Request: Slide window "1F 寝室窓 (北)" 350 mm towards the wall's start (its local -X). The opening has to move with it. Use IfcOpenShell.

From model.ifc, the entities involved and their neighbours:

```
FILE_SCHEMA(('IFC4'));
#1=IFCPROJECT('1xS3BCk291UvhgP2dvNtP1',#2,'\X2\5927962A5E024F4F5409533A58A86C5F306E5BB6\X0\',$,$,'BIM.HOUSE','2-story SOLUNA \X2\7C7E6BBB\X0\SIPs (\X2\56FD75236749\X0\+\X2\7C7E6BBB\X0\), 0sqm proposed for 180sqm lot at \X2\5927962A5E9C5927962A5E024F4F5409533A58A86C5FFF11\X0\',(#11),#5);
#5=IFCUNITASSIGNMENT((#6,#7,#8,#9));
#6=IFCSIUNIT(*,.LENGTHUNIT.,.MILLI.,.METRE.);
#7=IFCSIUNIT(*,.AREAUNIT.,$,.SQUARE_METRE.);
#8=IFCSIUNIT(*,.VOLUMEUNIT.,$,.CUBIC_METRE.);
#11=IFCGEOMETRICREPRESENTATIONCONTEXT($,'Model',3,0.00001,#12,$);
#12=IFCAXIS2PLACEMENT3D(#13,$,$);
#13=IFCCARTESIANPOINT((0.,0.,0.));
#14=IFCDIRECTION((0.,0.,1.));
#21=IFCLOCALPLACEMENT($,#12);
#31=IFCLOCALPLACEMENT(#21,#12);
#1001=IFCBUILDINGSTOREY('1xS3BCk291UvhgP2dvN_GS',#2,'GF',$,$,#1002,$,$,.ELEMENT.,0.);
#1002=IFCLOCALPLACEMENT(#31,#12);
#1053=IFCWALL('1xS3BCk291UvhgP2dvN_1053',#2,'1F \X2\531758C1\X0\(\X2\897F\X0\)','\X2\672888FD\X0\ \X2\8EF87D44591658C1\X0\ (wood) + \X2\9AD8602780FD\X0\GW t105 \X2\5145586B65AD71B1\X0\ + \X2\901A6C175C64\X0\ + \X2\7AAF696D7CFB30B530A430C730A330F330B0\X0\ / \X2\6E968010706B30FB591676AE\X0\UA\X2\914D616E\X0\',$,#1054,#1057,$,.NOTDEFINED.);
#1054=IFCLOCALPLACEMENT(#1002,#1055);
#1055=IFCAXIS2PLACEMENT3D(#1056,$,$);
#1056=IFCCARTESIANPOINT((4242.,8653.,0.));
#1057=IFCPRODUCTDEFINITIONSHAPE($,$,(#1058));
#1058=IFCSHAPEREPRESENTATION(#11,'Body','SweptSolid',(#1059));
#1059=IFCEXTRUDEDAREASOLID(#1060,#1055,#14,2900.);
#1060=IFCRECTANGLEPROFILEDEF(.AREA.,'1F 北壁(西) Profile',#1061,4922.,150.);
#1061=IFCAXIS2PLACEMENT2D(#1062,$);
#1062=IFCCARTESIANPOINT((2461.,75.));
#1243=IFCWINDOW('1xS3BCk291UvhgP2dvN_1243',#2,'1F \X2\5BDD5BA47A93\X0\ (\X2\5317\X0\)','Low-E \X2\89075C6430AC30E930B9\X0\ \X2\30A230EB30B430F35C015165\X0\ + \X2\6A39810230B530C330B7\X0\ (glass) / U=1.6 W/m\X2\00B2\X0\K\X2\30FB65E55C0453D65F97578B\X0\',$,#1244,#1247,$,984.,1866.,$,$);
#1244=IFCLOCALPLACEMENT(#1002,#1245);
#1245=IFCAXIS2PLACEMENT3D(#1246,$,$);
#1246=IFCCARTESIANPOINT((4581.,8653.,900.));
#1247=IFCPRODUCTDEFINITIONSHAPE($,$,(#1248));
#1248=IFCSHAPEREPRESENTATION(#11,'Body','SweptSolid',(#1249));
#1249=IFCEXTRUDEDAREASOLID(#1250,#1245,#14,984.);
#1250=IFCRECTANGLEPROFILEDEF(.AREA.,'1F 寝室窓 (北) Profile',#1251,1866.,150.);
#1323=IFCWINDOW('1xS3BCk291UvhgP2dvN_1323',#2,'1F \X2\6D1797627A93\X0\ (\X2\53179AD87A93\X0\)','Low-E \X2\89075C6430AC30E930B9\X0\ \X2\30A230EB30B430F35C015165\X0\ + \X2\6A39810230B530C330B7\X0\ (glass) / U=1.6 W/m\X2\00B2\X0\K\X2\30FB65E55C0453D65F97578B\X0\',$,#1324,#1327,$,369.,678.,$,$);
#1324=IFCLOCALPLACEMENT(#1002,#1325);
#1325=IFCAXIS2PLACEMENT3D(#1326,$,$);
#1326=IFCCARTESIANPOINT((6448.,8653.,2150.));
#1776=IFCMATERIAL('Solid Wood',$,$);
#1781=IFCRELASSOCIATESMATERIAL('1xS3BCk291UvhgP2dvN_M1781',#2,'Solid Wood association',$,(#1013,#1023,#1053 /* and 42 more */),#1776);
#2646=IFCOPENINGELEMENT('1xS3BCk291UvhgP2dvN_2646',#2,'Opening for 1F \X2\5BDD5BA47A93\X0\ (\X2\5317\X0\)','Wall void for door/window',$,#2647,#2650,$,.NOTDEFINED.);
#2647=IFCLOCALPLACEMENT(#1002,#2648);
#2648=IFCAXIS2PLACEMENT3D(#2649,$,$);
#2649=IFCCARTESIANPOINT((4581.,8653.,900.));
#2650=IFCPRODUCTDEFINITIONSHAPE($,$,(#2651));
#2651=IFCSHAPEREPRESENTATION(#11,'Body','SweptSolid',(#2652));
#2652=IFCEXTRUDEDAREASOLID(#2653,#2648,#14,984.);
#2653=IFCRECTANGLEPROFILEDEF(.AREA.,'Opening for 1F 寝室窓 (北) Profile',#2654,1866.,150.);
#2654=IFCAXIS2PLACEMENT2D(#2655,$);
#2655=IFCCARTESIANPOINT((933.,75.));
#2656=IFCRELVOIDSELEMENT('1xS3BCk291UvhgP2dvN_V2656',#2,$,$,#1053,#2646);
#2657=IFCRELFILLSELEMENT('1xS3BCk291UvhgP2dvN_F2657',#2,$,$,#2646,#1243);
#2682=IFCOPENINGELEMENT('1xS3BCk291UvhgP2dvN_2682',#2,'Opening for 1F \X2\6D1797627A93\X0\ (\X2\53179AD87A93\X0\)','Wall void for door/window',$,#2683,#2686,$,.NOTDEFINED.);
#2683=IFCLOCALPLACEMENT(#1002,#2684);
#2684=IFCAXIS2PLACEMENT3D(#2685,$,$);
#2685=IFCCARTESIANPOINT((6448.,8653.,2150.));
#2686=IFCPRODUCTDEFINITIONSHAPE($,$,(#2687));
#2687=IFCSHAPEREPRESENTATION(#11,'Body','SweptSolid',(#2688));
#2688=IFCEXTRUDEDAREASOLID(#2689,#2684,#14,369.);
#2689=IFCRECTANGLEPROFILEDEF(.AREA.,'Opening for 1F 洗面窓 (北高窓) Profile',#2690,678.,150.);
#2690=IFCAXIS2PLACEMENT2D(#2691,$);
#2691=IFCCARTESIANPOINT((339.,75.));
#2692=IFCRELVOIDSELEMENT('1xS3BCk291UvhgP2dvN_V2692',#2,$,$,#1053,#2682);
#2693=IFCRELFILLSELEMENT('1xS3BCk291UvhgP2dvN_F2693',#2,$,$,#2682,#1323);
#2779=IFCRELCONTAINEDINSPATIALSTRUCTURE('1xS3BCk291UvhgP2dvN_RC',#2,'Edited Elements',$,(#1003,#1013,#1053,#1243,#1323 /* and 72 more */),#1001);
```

```python
import ifcopenshell
import ifcopenshell.api.geometry
import ifcopenshell.util.placement

model = ifcopenshell.open("model.ifc")

window = model.by_guid("1xS3BCk291UvhgP2dvN_1243")
opening = window.FillsVoids[0].RelatingOpeningElement
wall = opening.VoidsElements[0].RelatingBuildingElement

wall_matrix = ifcopenshell.util.placement.get_local_placement(wall.ObjectPlacement)
shift = wall_matrix[:3, 0] * -350.0
before = ifcopenshell.util.placement.get_local_placement(window.ObjectPlacement)[:3, 3].copy()

# The window is not placed relative to its opening, so move both.
for product in (opening, window):
    matrix = ifcopenshell.util.placement.get_local_placement(product.ObjectPlacement)
    matrix[:3, 3] += shift
    ifcopenshell.api.geometry.edit_object_placement(model, product=product, matrix=matrix, is_si=False)

after = ifcopenshell.util.placement.get_local_placement(window.ObjectPlacement)[:3, 3]
print("window moved by", (after - before).round(3) + 0.0)

model.write("model_rev.ifc")
```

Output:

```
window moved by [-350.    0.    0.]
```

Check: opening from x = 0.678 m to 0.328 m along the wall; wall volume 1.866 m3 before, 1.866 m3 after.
